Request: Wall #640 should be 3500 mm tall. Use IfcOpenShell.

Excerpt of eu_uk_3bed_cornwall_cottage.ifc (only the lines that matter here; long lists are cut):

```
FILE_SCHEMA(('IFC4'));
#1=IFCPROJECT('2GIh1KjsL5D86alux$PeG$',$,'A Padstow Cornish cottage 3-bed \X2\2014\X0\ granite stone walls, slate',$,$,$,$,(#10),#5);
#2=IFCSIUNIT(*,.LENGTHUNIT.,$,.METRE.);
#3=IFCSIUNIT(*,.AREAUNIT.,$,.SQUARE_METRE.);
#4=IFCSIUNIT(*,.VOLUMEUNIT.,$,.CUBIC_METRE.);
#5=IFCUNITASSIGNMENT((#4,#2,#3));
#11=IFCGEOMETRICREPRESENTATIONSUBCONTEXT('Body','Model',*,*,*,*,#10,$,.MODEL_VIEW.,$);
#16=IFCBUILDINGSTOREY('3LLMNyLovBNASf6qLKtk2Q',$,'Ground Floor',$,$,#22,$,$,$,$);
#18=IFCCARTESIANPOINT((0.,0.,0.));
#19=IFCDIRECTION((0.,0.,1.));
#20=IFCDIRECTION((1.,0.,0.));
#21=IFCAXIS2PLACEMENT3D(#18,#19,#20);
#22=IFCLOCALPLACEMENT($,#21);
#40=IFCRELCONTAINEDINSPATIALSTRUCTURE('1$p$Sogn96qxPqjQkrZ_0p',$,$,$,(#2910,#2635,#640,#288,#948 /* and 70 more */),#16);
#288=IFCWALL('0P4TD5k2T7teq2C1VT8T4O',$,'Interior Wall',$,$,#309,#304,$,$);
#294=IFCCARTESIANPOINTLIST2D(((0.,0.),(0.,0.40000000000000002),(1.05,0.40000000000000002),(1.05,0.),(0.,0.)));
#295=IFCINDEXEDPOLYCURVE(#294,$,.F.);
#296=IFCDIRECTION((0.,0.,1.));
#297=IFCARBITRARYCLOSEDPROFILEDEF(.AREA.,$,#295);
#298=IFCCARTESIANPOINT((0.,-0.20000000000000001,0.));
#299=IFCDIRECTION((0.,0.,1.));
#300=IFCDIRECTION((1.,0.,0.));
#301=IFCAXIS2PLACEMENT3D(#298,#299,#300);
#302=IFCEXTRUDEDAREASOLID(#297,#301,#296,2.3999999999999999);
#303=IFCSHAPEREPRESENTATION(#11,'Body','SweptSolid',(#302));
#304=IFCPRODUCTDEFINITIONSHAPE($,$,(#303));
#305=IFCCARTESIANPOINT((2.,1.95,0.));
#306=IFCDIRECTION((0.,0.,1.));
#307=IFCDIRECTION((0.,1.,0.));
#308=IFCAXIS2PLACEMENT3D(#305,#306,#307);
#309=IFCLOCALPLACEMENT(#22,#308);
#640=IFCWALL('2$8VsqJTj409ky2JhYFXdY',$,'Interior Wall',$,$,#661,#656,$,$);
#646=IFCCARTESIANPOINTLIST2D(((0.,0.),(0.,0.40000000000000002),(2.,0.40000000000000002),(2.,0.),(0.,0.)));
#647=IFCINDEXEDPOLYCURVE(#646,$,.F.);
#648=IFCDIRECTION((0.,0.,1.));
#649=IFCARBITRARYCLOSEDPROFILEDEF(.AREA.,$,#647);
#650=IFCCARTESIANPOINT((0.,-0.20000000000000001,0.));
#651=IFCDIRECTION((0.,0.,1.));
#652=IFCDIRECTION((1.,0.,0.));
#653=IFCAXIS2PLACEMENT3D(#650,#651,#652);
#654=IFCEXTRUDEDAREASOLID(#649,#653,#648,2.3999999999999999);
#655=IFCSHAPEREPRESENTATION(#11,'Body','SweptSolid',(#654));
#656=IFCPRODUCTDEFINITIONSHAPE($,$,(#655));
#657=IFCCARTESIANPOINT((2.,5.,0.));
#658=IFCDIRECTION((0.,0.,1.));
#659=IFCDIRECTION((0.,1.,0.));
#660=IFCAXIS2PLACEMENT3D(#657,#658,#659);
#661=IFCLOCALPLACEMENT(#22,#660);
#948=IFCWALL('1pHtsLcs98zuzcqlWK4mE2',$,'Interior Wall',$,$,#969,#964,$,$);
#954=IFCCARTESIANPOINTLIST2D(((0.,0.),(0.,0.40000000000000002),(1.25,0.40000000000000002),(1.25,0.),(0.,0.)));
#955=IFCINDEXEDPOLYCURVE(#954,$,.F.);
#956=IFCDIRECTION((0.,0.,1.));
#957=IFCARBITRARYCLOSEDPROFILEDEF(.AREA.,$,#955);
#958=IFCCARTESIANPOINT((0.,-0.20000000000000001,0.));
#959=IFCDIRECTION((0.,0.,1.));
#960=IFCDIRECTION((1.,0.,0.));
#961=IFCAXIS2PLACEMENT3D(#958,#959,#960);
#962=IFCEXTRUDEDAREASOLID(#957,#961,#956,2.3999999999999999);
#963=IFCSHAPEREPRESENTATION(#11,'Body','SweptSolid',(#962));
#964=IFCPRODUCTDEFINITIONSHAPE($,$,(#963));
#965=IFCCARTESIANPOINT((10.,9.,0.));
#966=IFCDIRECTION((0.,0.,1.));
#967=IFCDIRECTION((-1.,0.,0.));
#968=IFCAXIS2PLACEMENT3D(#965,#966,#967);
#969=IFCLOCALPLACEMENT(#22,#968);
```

```python
import ifcopenshell
import ifcopenshell.geom
import ifcopenshell.util.representation
import ifcopenshell.util.shape

model = ifcopenshell.open("eu_uk_3bed_cornwall_cottage.ifc")
settings = ifcopenshell.geom.settings()


def volume(element):
    """Net volume in cubic metres, openings subtracted."""
    shape = ifcopenshell.geom.create_shape(settings, element)
    return ifcopenshell.util.shape.get_volume(shape.geometry)


wall = model.by_guid("2$8VsqJTj409ky2JhYFXdY")
before = volume(wall)

body = ifcopenshell.util.representation.get_representation(wall, "Model", "Body")
solid = body.Items[0]
old_height = solid.Depth
solid.Depth = 3.5
after = volume(wall)

print(f"height {old_height:g} -> {solid.Depth:g}, volume {before:.3f} -> {after:.3f} m3")

model.write("eu_uk_3bed_cornwall_cottage_edited.ifc")
```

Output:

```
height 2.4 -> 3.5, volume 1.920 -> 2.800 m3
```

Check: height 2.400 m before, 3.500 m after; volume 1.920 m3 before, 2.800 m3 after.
